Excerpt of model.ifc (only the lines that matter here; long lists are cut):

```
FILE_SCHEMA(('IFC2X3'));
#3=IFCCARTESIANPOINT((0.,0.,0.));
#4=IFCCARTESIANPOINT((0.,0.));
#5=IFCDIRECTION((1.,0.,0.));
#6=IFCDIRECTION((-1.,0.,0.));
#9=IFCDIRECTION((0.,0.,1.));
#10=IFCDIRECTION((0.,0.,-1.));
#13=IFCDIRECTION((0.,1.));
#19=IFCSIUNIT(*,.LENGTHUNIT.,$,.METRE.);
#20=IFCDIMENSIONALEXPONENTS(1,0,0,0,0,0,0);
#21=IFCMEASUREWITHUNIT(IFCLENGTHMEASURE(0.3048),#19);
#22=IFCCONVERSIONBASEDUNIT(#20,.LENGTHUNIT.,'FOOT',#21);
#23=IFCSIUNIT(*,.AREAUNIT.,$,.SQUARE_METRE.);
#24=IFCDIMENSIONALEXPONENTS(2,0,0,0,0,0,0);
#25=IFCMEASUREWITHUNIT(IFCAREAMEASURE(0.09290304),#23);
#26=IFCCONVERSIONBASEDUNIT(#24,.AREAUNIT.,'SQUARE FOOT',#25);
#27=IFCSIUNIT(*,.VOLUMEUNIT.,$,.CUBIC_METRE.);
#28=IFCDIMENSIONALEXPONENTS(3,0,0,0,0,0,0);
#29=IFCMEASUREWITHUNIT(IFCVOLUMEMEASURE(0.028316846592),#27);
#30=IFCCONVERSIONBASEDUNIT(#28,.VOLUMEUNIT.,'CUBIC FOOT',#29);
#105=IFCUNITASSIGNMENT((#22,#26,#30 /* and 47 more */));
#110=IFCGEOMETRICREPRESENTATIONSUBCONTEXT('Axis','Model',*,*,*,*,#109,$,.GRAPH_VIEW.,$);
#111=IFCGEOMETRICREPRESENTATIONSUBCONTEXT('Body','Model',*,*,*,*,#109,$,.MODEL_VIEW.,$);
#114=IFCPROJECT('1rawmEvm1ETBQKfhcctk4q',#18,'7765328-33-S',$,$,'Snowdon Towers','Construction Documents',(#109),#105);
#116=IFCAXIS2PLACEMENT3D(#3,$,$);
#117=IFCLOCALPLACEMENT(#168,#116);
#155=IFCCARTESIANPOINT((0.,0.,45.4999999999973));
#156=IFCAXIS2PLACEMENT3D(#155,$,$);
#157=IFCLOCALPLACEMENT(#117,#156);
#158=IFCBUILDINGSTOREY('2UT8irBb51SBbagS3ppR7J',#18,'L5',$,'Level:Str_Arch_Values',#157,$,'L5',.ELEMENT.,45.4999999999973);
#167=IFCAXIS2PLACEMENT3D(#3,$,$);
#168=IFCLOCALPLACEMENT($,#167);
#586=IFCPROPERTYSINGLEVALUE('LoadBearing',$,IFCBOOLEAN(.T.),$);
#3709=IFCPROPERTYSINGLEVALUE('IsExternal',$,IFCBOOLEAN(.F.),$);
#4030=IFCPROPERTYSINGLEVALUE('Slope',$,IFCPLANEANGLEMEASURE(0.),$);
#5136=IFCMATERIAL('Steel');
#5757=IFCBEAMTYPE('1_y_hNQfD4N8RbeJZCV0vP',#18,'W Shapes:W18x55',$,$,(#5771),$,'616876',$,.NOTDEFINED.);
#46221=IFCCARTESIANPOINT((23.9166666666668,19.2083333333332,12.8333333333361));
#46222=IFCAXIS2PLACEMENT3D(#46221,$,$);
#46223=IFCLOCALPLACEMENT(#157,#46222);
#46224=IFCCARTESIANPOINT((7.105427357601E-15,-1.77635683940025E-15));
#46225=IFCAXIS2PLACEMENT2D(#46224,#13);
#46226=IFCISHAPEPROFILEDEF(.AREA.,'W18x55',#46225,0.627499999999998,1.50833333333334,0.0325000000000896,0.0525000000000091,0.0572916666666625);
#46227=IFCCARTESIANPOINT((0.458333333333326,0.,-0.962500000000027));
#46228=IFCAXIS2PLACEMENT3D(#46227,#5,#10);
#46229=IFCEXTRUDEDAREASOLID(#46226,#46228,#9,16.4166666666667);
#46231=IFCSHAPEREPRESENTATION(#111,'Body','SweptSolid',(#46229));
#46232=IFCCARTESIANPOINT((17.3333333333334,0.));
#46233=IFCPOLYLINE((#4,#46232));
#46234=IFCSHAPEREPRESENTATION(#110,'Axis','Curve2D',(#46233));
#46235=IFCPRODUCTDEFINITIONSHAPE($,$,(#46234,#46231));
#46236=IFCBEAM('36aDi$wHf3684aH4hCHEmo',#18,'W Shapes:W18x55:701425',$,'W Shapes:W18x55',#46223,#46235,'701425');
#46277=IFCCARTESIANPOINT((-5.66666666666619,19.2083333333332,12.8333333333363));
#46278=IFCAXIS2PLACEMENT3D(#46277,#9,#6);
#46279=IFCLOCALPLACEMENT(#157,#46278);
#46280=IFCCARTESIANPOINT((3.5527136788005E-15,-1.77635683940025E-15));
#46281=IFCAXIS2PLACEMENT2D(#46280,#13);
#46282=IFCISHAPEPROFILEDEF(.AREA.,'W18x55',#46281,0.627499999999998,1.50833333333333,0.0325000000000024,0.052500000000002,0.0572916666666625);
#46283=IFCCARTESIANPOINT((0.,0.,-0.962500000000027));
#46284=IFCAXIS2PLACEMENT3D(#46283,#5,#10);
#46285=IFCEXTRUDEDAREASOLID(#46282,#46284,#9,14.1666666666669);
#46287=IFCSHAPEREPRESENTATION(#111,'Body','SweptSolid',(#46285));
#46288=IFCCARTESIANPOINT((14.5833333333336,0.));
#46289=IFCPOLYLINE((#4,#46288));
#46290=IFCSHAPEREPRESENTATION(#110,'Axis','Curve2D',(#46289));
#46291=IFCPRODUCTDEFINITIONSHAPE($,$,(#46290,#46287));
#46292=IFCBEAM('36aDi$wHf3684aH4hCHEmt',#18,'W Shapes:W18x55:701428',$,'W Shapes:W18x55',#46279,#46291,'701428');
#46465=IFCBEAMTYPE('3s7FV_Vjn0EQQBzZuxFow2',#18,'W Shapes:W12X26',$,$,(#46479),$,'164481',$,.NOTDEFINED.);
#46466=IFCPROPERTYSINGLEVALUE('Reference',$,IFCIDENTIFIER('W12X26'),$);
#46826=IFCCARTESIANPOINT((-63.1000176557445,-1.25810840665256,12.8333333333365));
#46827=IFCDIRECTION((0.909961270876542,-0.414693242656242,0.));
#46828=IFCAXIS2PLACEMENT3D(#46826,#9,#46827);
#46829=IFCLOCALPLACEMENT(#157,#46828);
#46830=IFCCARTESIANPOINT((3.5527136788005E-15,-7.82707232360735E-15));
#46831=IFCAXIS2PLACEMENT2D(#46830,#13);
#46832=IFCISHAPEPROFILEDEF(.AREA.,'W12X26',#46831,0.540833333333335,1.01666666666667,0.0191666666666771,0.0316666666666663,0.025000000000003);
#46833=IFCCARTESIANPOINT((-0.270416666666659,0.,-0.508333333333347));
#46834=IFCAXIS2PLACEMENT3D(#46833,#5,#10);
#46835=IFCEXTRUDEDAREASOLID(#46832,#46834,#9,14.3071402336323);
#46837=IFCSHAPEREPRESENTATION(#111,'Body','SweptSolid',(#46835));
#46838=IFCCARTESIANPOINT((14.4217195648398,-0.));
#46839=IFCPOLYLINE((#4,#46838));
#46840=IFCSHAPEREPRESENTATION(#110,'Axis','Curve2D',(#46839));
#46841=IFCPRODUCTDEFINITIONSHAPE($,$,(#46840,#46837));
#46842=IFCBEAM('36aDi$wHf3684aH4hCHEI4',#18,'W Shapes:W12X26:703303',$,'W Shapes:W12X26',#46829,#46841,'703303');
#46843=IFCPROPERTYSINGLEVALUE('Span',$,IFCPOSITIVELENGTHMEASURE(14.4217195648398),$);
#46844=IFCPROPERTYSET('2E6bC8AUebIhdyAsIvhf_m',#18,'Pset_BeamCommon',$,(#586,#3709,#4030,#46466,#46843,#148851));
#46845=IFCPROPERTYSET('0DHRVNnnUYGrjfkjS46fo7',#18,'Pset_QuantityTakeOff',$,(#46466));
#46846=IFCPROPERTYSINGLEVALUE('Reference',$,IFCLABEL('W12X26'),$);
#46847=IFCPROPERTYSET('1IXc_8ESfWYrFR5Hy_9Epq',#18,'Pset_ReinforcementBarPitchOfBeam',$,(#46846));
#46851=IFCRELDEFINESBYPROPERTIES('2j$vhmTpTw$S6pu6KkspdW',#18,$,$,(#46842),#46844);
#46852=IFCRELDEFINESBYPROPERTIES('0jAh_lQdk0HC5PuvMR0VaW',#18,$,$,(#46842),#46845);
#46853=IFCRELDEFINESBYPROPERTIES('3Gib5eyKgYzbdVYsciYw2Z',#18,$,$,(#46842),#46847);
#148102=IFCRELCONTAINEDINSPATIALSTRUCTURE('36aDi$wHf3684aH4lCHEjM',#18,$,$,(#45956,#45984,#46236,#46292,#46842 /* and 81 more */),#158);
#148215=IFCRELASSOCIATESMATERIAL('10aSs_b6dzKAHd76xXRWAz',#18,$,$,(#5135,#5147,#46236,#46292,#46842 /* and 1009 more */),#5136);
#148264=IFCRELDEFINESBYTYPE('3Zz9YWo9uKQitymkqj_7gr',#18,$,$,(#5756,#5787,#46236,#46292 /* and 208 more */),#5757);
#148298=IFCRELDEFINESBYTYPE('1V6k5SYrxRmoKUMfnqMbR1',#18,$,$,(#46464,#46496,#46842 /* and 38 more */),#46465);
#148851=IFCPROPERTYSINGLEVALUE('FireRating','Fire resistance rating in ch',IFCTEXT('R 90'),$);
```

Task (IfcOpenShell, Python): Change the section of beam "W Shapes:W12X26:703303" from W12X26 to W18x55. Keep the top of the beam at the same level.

```python
import ifcopenshell
import ifcopenshell.api.pset
import ifcopenshell.api.type
import ifcopenshell.util.element
import ifcopenshell.util.representation

model = ifcopenshell.open("model.ifc")

member = model.by_guid("36aDi$wHf3684aH4hCHEI4")
source = next(p for p in model.by_type("IfcIShapeProfileDef") if p.ProfileName == "W18x55")

body = ifcopenshell.util.representation.get_representation(member, "Model", "Body")
solid = body.Items[0]
old_profile = solid.SweptArea

# Copy the section's sizes but keep this member's own profile position.
profile = ifcopenshell.util.element.copy(model, source)
# Profiles are centred, so shift by half the change in depth to hold the top.
shift = (old_profile.OverallDepth - profile.OverallDepth) / 2
x, y = old_profile.Position.Location.Coordinates
up = (-1.0, 0.0)  # upwards, in the solid's own plane
location = model.createIfcCartesianPoint((x + up[0] * shift, y + up[1] * shift))
profile.Position = model.createIfcAxis2Placement2D(location, old_profile.Position.RefDirection)
solid.SweptArea = profile
if not model.get_total_inverses(old_profile):
    ifcopenshell.util.element.remove_deep2(model, old_profile)

new_type = model.by_guid("1_y_hNQfD4N8RbeJZCV0vP")
ifcopenshell.api.type.assign_type(
    model, related_objects=[member], relating_type=new_type, should_map_representations=False
)
member.Name = member.Name.replace("W12X26", "W18x55")
member.ObjectType = "W Shapes:W18x55"
pset = model.by_id(ifcopenshell.util.element.get_pset(member, "Pset_BeamCommon", should_inherit=False)["id"])
ifcopenshell.api.pset.edit_pset(model, pset=pset, properties={"Reference": "W18x55"})
pset = model.by_id(ifcopenshell.util.element.get_pset(member, "Pset_QuantityTakeOff", should_inherit=False)["id"])
ifcopenshell.api.pset.edit_pset(model, pset=pset, properties={"Reference": "W18x55"})
pset = model.by_id(ifcopenshell.util.element.get_pset(member, "Pset_ReinforcementBarPitchOfBeam", should_inherit=False)["id"])
ifcopenshell.api.pset.edit_pset(model, pset=pset, properties={"Reference": "W18x55"})

print(solid.SweptArea)

model.write("model_v2.ifc")
```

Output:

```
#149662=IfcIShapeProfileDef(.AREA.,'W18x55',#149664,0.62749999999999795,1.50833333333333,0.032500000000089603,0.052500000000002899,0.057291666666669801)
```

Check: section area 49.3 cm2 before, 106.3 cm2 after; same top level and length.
